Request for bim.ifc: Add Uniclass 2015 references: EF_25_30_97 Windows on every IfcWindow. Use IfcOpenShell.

First a look at what the model holds.

```python
import ifcopenshell

model = ifcopenshell.open("bim.ifc")
print(model.schema)
print("classifications:", [c.Name for c in model.by_type("IfcClassification")])
for ifc_class in ("IfcDoor", "IfcRoof", "IfcStair", "IfcWall", "IfcWindow"):
    print(ifc_class, len(model.by_type(ifc_class)))
```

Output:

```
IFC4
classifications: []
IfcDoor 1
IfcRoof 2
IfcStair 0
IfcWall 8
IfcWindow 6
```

```python
import ifcopenshell
import ifcopenshell.api.classification

model = ifcopenshell.open("bim.ifc")

system = ifcopenshell.api.classification.add_classification(model, classification="Uniclass 2015")

codes = {
    "IfcWindow": ("EF_25_30_97", "Windows"),
}
for ifc_class, (code, name) in codes.items():
    products = model.by_type(ifc_class)
    ifcopenshell.api.classification.add_reference(
        model, products=products, classification=system, identification=code, name=name
    )
    print(code, len(products))

model.write("bim-out.ifc")
```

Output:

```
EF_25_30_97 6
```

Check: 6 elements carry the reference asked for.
